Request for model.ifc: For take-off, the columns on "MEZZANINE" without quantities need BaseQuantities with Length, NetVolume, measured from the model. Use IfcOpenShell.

First a look at what the model holds.

```python
import ifcopenshell
import ifcopenshell.util.element
import ifcopenshell.util.unit

model = ifcopenshell.open("model.ifc")
print(model.schema)
for unit_type in ("LENGTHUNIT", "AREAUNIT", "VOLUMEUNIT"):
    print(unit_type, ifcopenshell.util.unit.calculate_unit_scale(model, unit_type))
storey = next(s for s in model.by_type("IfcBuildingStorey") if s.Name == "MEZZANINE")
columns = [e for e in ifcopenshell.util.element.get_decomposition(storey) if e.is_a("IfcColumn")]
for e in sorted(columns, key=lambda e: e.id()):
    print(e.id(), e.is_a(), e.Name, list(ifcopenshell.util.element.get_psets(e, qtos_only=True)), sep=" | ")
```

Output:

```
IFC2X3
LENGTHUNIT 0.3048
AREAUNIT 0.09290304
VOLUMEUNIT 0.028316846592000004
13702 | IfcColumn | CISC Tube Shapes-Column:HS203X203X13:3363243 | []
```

```python
import ifcopenshell
import ifcopenshell.api.pset
import ifcopenshell.geom
import ifcopenshell.util.element
import ifcopenshell.util.shape
import ifcopenshell.util.unit

model = ifcopenshell.open("model.ifc")
unit_scale = ifcopenshell.util.unit.calculate_unit_scale(model)
volume_scale = ifcopenshell.util.unit.calculate_unit_scale(model, "VOLUMEUNIT")
settings = ifcopenshell.geom.settings()

storey = next(s for s in model.by_type("IfcBuildingStorey") if s.Name == "MEZZANINE")
columns = [e for e in ifcopenshell.util.element.get_decomposition(storey) if e.is_a("IfcColumn")]

for e in sorted(columns, key=lambda e: e.id()):
    if ifcopenshell.util.element.get_psets(e, qtos_only=True, should_inherit=False):
        continue
    # Geometry comes back in metres, in the element's own axes.
    shape = ifcopenshell.geom.create_shape(settings, e)
    values = {
        "Length": ifcopenshell.util.shape.get_z(shape.geometry) / unit_scale,
        "NetVolume": ifcopenshell.util.shape.get_volume(shape.geometry) / volume_scale,
    }
    qto = ifcopenshell.api.pset.add_qto(model, product=e, name="BaseQuantities")
    ifcopenshell.api.pset.edit_qto(model, qto=qto, properties=values)
    print(e.id(), {k: round(v, 3) for k, v in values.items()})

model.write("model_v2.ifc")
```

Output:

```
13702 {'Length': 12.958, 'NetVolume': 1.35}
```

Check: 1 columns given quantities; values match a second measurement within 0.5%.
